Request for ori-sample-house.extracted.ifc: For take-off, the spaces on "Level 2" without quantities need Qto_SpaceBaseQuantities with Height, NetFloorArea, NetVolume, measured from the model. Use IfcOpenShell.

First a look at what the model holds.

```python
import ifcopenshell
import ifcopenshell.util.element
import ifcopenshell.util.unit

model = ifcopenshell.open("ori-sample-house.extracted.ifc")
print(model.schema)
for unit_type in ("LENGTHUNIT", "AREAUNIT", "VOLUMEUNIT"):
    print(unit_type, ifcopenshell.util.unit.calculate_unit_scale(model, unit_type))
storey = next(s for s in model.by_type("IfcBuildingStorey") if s.Name == "Level 2")
spaces = [e for e in ifcopenshell.util.element.get_decomposition(storey) if e.is_a("IfcSpace")]
for e in sorted(spaces, key=lambda e: e.id()):
    print(e.id(), e.is_a(), e.Name, list(ifcopenshell.util.element.get_psets(e, qtos_only=True)), sep=" | ")
```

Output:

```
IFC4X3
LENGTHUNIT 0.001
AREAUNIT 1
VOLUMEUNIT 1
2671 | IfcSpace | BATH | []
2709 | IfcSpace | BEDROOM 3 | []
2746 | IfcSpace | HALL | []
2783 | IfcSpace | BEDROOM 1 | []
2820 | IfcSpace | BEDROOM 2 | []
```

```python
import ifcopenshell
import ifcopenshell.api.pset
import ifcopenshell.geom
import ifcopenshell.util.element
import ifcopenshell.util.shape
import ifcopenshell.util.unit

model = ifcopenshell.open("ori-sample-house.extracted.ifc")
unit_scale = ifcopenshell.util.unit.calculate_unit_scale(model)
area_scale = ifcopenshell.util.unit.calculate_unit_scale(model, "AREAUNIT")
volume_scale = ifcopenshell.util.unit.calculate_unit_scale(model, "VOLUMEUNIT")
settings = ifcopenshell.geom.settings()

storey = next(s for s in model.by_type("IfcBuildingStorey") if s.Name == "Level 2")
spaces = [e for e in ifcopenshell.util.element.get_decomposition(storey) if e.is_a("IfcSpace")]

for e in sorted(spaces, key=lambda e: e.id()):
    if ifcopenshell.util.element.get_psets(e, qtos_only=True, should_inherit=False):
        continue
    # Geometry comes back in metres, in the element's own axes.
    shape = ifcopenshell.geom.create_shape(settings, e)
    values = {
        "Height": ifcopenshell.util.shape.get_z(shape.geometry) / unit_scale,
        "NetFloorArea": ifcopenshell.util.shape.get_footprint_area(shape.geometry) / area_scale,
        "NetVolume": ifcopenshell.util.shape.get_volume(shape.geometry) / volume_scale,
    }
    qto = ifcopenshell.api.pset.add_qto(model, product=e, name="Qto_SpaceBaseQuantities")
    ifcopenshell.api.pset.edit_qto(model, qto=qto, properties=values)
    print(e.id(), {k: round(v, 3) for k, v in values.items()})

model.write("ori-sample-house.extracted_rev.ifc")
```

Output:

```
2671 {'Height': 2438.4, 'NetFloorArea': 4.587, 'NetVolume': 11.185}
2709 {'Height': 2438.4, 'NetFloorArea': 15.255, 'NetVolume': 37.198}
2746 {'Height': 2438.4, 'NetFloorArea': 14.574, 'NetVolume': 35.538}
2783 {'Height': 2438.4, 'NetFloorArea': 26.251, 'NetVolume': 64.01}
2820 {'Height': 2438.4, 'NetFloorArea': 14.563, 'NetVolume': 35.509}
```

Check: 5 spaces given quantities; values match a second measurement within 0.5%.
